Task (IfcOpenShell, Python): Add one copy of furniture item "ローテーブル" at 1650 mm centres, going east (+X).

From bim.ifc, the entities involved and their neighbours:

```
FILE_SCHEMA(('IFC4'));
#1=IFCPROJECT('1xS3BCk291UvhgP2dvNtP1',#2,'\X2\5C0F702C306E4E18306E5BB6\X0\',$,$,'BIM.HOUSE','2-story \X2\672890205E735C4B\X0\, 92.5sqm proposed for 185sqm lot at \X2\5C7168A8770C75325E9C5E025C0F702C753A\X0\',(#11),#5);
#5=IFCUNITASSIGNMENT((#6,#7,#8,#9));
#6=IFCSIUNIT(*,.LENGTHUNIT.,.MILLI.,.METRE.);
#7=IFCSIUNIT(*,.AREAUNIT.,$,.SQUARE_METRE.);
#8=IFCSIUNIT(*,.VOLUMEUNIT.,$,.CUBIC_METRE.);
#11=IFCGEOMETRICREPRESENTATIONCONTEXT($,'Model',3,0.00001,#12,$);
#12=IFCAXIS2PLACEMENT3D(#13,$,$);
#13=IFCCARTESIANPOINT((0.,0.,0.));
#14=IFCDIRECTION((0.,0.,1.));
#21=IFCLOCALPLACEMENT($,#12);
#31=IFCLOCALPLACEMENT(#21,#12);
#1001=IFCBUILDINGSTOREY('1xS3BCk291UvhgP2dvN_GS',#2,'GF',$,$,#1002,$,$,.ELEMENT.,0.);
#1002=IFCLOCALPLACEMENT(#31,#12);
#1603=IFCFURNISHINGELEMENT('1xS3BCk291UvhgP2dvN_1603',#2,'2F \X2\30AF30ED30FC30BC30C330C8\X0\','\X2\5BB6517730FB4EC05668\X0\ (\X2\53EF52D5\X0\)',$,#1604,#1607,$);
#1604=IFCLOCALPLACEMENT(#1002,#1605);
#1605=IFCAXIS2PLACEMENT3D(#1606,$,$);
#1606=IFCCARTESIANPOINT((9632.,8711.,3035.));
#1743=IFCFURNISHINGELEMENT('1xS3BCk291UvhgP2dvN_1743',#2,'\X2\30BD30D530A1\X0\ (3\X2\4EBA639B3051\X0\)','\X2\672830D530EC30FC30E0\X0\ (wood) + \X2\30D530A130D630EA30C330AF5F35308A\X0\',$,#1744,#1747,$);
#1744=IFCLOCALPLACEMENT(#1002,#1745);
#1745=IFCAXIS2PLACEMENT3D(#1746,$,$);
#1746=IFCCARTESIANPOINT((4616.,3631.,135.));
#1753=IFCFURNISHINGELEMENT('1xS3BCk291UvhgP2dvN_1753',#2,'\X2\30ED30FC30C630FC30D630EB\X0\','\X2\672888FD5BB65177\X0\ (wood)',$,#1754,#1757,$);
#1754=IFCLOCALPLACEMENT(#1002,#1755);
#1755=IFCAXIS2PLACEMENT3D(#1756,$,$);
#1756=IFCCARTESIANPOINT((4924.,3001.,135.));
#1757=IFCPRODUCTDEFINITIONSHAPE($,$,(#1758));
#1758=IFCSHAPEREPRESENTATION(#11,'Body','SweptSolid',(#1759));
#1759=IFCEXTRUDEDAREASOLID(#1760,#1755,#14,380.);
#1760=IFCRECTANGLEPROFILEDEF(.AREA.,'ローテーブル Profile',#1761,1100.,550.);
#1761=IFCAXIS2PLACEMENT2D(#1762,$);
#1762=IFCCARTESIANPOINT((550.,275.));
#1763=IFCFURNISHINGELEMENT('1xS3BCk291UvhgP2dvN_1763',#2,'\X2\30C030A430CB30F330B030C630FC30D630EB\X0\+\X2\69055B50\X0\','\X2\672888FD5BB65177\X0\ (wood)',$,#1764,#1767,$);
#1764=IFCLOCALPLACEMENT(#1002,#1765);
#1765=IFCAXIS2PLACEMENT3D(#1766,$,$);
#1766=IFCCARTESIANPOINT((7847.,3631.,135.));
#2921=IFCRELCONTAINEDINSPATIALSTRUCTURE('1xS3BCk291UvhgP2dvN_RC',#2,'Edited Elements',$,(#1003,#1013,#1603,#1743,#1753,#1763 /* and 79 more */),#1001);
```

```python
import numpy as np
import ifcopenshell
import ifcopenshell.api.geometry
import ifcopenshell.api.root
import ifcopenshell.util.element
import ifcopenshell.util.placement

model = ifcopenshell.open("bim.ifc")


def reuse_history(source, copy):
    """copy_class also copies each property set's owner history, people and application; keep the originals."""
    for rel in copy.IsDefinedBy:
        if rel.is_a("IfcRelDefinesByProperties") and (history := rel.RelatingPropertyDefinition.OwnerHistory):
            rel.RelatingPropertyDefinition.OwnerHistory = source.OwnerHistory
            ifcopenshell.util.element.remove_deep2(model, history)


source = model.by_guid("1xS3BCk291UvhgP2dvN_1753")
base = ifcopenshell.util.placement.get_local_placement(source.ObjectPlacement)
step = np.array([1.0, 0.0, 0.0]) * 1650.0

for i in range(1, 2):
    copy = ifcopenshell.api.root.copy_class(model, product=source)
    copy.Representation = ifcopenshell.util.element.copy_deep(
        model, source.Representation, exclude=["IfcGeometricRepresentationContext", "IfcRepresentationMap"]
    )
    reuse_history(source, copy)
    matrix = base.copy()
    matrix[:3, 3] += i * step
    print("added at", matrix[:3, 3].round(3) + 0.0)
    ifcopenshell.api.geometry.edit_object_placement(model, product=copy, matrix=matrix, is_si=False)

model.write("bim_rev.ifc")
```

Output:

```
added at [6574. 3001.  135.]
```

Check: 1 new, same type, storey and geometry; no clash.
